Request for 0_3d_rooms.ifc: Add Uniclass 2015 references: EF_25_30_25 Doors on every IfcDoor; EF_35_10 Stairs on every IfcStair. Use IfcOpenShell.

First a look at what the model holds.

```python
import ifcopenshell

model = ifcopenshell.open("0_3d_rooms.ifc")
print(model.schema)
print("classifications:", [c.Name for c in model.by_type("IfcClassification")])
for ifc_class in ("IfcDoor", "IfcRoof", "IfcStair", "IfcWall", "IfcWindow"):
    print(ifc_class, len(model.by_type(ifc_class)))
```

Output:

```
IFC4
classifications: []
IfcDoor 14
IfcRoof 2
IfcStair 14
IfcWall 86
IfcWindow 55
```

```python
import ifcopenshell
import ifcopenshell.api.classification

model = ifcopenshell.open("0_3d_rooms.ifc")

system = ifcopenshell.api.classification.add_classification(model, classification="Uniclass 2015")

codes = {
    "IfcDoor": ("EF_25_30_25", "Doors"),
    "IfcStair": ("EF_35_10", "Stairs"),
}
for ifc_class, (code, name) in codes.items():
    products = model.by_type(ifc_class)
    ifcopenshell.api.classification.add_reference(
        model, products=products, classification=system, identification=code, name=name
    )
    print(code, len(products))

model.write("0_3d_rooms_rev.ifc")
```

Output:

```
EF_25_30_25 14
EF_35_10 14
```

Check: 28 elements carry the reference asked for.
